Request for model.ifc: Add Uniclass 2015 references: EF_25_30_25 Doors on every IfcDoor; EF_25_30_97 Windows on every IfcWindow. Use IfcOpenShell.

First a look at what the model holds.

```python
import ifcopenshell

model = ifcopenshell.open("model.ifc")
print(model.schema)
print("classifications:", [c.Name for c in model.by_type("IfcClassification")])
for ifc_class in ("IfcDoor", "IfcRoof", "IfcStair", "IfcWall", "IfcWindow"):
    print(ifc_class, len(model.by_type(ifc_class)))
```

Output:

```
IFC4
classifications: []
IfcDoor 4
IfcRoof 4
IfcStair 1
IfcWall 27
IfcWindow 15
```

```python
import ifcopenshell
import ifcopenshell.api.classification

model = ifcopenshell.open("model.ifc")

system = ifcopenshell.api.classification.add_classification(model, classification="Uniclass 2015")

codes = {
    "IfcDoor": ("EF_25_30_25", "Doors"),
    "IfcWindow": ("EF_25_30_97", "Windows"),
}
for ifc_class, (code, name) in codes.items():
    products = model.by_type(ifc_class)
    ifcopenshell.api.classification.add_reference(
        model, products=products, classification=system, identification=code, name=name
    )
    print(code, len(products))

model.write("model_edited.ifc")
```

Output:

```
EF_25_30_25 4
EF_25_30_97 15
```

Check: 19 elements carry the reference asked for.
